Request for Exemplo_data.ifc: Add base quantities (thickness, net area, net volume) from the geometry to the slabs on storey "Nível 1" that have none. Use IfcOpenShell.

First a look at what the model holds.

```python
import ifcopenshell
import ifcopenshell.util.element
import ifcopenshell.util.unit

model = ifcopenshell.open("Exemplo_data.ifc")
print(model.schema)
for unit_type in ("LENGTHUNIT", "AREAUNIT", "VOLUMEUNIT"):
    print(unit_type, ifcopenshell.util.unit.calculate_unit_scale(model, unit_type))
storey = next(s for s in model.by_type("IfcBuildingStorey") if s.Name == "Nível 1")
slabs = [e for e in ifcopenshell.util.element.get_decomposition(storey) if e.is_a("IfcSlab")]
for e in sorted(slabs, key=lambda e: e.id()):
    print(e.id(), e.is_a(), e.Name, list(ifcopenshell.util.element.get_psets(e, qtos_only=True)), sep=" | ")
```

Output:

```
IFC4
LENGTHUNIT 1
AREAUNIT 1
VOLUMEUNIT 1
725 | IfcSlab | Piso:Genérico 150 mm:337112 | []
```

```python
import ifcopenshell
import ifcopenshell.api.pset
import ifcopenshell.geom
import ifcopenshell.util.element
import ifcopenshell.util.shape
import ifcopenshell.util.unit

model = ifcopenshell.open("Exemplo_data.ifc")
unit_scale = ifcopenshell.util.unit.calculate_unit_scale(model)
area_scale = ifcopenshell.util.unit.calculate_unit_scale(model, "AREAUNIT")
volume_scale = ifcopenshell.util.unit.calculate_unit_scale(model, "VOLUMEUNIT")
settings = ifcopenshell.geom.settings()

storey = next(s for s in model.by_type("IfcBuildingStorey") if s.Name == "Nível 1")
slabs = [e for e in ifcopenshell.util.element.get_decomposition(storey) if e.is_a("IfcSlab")]

for e in sorted(slabs, key=lambda e: e.id()):
    if ifcopenshell.util.element.get_psets(e, qtos_only=True, should_inherit=False):
        continue
    # Geometry comes back in metres, in the element's own axes.
    shape = ifcopenshell.geom.create_shape(settings, e)
    values = {
        "Width": ifcopenshell.util.shape.get_z(shape.geometry) / unit_scale,
        "NetArea": ifcopenshell.util.shape.get_footprint_area(shape.geometry) / area_scale,
        "NetVolume": ifcopenshell.util.shape.get_volume(shape.geometry) / volume_scale,
    }
    qto = ifcopenshell.api.pset.add_qto(model, product=e, name="Qto_SlabBaseQuantities")
    ifcopenshell.api.pset.edit_qto(model, qto=qto, properties=values)
    print(e.id(), {k: round(v, 3) for k, v in values.items()})

model.write("Exemplo_data_v2.ifc")
```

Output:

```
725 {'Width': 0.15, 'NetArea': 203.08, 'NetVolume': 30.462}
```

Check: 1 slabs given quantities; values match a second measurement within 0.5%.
